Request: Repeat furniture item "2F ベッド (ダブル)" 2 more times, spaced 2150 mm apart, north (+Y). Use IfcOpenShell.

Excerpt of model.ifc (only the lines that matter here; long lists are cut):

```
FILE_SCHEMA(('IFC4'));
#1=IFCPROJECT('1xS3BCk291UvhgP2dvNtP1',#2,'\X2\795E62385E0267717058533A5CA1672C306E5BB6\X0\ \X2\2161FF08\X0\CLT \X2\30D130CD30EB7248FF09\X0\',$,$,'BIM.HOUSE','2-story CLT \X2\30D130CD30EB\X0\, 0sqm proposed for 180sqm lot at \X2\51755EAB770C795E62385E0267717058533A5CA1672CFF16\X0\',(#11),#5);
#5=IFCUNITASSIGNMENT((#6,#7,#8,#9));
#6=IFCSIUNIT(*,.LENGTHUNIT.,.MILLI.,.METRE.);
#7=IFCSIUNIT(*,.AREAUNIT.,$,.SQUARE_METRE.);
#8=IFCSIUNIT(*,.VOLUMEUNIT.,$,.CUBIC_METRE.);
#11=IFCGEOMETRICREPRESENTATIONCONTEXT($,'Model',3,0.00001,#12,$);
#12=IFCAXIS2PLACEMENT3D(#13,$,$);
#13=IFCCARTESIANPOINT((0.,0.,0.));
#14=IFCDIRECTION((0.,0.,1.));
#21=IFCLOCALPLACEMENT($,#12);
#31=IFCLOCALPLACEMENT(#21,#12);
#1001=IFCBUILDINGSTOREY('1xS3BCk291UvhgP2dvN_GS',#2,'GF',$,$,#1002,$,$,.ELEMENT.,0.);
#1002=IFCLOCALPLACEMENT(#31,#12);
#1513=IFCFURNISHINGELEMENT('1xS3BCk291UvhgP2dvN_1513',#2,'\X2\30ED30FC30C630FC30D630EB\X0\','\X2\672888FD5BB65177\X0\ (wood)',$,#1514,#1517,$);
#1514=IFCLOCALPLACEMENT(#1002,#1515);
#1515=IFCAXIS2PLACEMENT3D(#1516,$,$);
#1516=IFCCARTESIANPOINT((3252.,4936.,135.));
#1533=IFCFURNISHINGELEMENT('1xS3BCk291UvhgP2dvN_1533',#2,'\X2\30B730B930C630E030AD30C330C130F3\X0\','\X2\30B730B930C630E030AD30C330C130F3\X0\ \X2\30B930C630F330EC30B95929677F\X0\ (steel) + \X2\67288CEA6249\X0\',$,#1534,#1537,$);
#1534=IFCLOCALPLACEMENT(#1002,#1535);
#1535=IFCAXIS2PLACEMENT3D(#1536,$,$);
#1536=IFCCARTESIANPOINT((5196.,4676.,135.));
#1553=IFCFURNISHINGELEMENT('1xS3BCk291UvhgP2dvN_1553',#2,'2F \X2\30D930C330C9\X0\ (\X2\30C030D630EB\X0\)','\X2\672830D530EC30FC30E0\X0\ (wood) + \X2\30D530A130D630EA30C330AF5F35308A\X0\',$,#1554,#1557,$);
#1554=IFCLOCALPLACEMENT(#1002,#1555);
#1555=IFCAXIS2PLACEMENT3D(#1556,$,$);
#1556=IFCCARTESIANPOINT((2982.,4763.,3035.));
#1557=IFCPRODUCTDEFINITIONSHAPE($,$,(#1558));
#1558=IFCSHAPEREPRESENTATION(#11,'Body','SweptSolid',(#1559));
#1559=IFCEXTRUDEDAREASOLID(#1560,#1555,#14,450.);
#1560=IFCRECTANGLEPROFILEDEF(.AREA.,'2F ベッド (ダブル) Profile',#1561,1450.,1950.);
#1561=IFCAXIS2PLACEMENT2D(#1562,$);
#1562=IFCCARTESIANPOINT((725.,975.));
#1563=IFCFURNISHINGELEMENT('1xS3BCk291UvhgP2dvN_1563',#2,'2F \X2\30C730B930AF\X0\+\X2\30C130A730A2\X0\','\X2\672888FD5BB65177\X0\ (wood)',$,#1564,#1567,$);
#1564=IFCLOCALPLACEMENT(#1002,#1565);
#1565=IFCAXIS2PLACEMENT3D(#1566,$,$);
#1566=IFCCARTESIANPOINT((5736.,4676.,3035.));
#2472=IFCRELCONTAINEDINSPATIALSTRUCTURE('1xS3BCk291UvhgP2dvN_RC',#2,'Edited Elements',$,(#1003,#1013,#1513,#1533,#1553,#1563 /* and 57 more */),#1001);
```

```python
import numpy as np
import ifcopenshell
import ifcopenshell.api.geometry
import ifcopenshell.api.root
import ifcopenshell.util.element
import ifcopenshell.util.placement
import ifcopenshell.util.unit

model = ifcopenshell.open("model.ifc")
unit_scale = ifcopenshell.util.unit.calculate_unit_scale(model)


def reuse_history(source, copy):
    """copy_class also copies each property set's owner history, people and application; keep the originals."""
    for rel in copy.IsDefinedBy:
        if rel.is_a("IfcRelDefinesByProperties") and (history := rel.RelatingPropertyDefinition.OwnerHistory):
            rel.RelatingPropertyDefinition.OwnerHistory = source.OwnerHistory
            ifcopenshell.util.element.remove_deep2(model, history)


source = model.by_id(1553)
base = ifcopenshell.util.placement.get_local_placement(source.ObjectPlacement)
step = np.array([0.0, 1.0, 0.0]) * 2.15 / unit_scale

for i in range(1, 3):
    copy = ifcopenshell.api.root.copy_class(model, product=source)
    copy.Representation = ifcopenshell.util.element.copy_deep(
        model, source.Representation, exclude=["IfcGeometricRepresentationContext", "IfcRepresentationMap"]
    )
    reuse_history(source, copy)
    matrix = base.copy()
    matrix[:3, 3] += i * step
    print("added at", matrix[:3, 3].round(3) + 0.0)
    ifcopenshell.api.geometry.edit_object_placement(model, product=copy, matrix=matrix, is_si=False)

model.write("model_updated.ifc")
```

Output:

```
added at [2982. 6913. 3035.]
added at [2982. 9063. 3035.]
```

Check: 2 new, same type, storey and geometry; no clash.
